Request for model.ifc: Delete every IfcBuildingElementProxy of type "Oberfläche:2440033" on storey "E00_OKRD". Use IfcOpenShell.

First a look at what the model holds.

```python
import ifcopenshell
import ifcopenshell.util.element

model = ifcopenshell.open("model.ifc")
print(model.schema)
storey = next(s for s in model.by_type("IfcBuildingStorey") if s.Name == "E00_OKRD")
proxies = [e for e in ifcopenshell.util.element.get_decomposition(storey) if e.is_a("IfcBuildingElementProxy")]
seen = {}
for e in proxies:
    element_type = ifcopenshell.util.element.get_type(e)
    name = element_type.Name if element_type not in (None, e) else None
    seen[name] = seen.get(name, 0) + 1
for name, count in sorted(seen.items(), key=str):
    print(count, "x", name)
```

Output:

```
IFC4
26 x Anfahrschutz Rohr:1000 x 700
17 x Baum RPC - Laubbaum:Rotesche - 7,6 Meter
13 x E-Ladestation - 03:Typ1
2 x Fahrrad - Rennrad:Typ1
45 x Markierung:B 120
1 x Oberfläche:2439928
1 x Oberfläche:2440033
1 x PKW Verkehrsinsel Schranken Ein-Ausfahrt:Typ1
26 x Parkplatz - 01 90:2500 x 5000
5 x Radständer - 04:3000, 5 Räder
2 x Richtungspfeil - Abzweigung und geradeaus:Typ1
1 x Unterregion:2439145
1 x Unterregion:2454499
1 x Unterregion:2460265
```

```python
import ifcopenshell
import ifcopenshell.api.root
import ifcopenshell.util.element

model = ifcopenshell.open("model.ifc")

storey = next(s for s in model.by_type("IfcBuildingStorey") if s.Name == "E00_OKRD")
proxies = [e for e in ifcopenshell.util.element.get_decomposition(storey) if e.is_a("IfcBuildingElementProxy")]
targets = [e for e in proxies if (t := ifcopenshell.util.element.get_type(e)) not in (None, e) and t.Name == "Oberfläche:2440033"]

for e in targets:
    ifcopenshell.api.root.remove_product(model, product=e)
print(len(targets), "removed")

model.write("model-out.ifc")
```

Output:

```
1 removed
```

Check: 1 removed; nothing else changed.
